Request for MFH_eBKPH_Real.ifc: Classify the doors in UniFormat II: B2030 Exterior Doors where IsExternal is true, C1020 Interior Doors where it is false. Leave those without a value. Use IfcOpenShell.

First a look at what the model holds.

```python
import ifcopenshell
import ifcopenshell.util.element

model = ifcopenshell.open("MFH_eBKPH_Real.ifc")
print(model.schema)
print("classifications:", [c.Name for c in model.by_type("IfcClassification")])
values = [ifcopenshell.util.element.get_pset(e, "Pset_DoorCommon", "IsExternal") for e in model.by_type("IfcDoor")]
for value in (True, False, None):
    print("IsExternal", value, values.count(value))
```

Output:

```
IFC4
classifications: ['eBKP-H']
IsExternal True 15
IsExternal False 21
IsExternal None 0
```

```python
import ifcopenshell
import ifcopenshell.api.classification
import ifcopenshell.util.element

model = ifcopenshell.open("MFH_eBKPH_Real.ifc")

system = ifcopenshell.api.classification.add_classification(model, classification="UniFormat II")

doors = model.by_type("IfcDoor")
external = {e: ifcopenshell.util.element.get_pset(e, "Pset_DoorCommon", "IsExternal") for e in doors}
for flag, code, name in ((True, "B2030", "Exterior Doors"), (False, "C1020", "Interior Doors")):
    products = [e for e in doors if external[e] is flag]
    ifcopenshell.api.classification.add_reference(
        model, products=products, classification=system, identification=code, name=name
    )
    print(code, len(products))

model.write("MFH_eBKPH_Real_v2.ifc")
```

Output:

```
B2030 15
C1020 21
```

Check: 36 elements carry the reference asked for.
